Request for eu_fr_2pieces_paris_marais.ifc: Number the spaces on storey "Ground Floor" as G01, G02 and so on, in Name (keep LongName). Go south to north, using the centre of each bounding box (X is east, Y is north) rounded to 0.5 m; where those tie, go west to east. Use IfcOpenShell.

First a look at what the model holds.

```python
import ifcopenshell
import ifcopenshell.util.element
import ifcopenshell.util.placement

model = ifcopenshell.open("eu_fr_2pieces_paris_marais.ifc")
print(model.schema)
storey = next(s for s in model.by_type("IfcBuildingStorey") if s.Name == "Ground Floor")
spaces = [e for e in ifcopenshell.util.element.get_decomposition(storey) if e.is_a("IfcSpace")]
for e in sorted(spaces, key=lambda e: e.id()):
    origin = ifcopenshell.util.placement.get_local_placement(e.ObjectPlacement)[:3, 3]
    print(e.id(), e.Name, e.LongName, origin.round(2) + 0.0, sep=" | ")
```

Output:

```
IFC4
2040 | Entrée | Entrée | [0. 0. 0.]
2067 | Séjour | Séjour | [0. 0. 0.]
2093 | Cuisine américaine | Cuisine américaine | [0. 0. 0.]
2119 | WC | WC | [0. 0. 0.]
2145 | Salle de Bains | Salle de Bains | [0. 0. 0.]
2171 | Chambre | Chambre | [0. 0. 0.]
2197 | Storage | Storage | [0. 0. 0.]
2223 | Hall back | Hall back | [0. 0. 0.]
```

```python
import ifcopenshell
import ifcopenshell.geom
import ifcopenshell.util.element
import ifcopenshell.util.shape

model = ifcopenshell.open("eu_fr_2pieces_paris_marais.ifc")
settings = ifcopenshell.geom.settings()
settings.set("use-world-coords", True)


def centre(element):
    shape = ifcopenshell.geom.create_shape(settings, element)
    return ifcopenshell.util.shape.get_bbox_centroid(shape.geometry)


storey = next(s for s in model.by_type("IfcBuildingStorey") if s.Name == "Ground Floor")
spaces = [e for e in ifcopenshell.util.element.get_decomposition(storey) if e.is_a("IfcSpace")]

# Insertion points can sit at a corner or the storey origin, so sort by the geometry (in metres).
centres = {e: centre(e) for e in spaces}
spaces.sort(key=lambda e: (round(centres[e][1] / 0.5), centres[e][0]))

for i, e in enumerate(spaces, start=1):
    number = f"G{i:02d}"
    e.Name = number
    print(e.id(), number)

model.write("eu_fr_2pieces_paris_marais-out.ifc")
```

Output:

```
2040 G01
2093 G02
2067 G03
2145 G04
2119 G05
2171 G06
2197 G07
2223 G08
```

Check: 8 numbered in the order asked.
